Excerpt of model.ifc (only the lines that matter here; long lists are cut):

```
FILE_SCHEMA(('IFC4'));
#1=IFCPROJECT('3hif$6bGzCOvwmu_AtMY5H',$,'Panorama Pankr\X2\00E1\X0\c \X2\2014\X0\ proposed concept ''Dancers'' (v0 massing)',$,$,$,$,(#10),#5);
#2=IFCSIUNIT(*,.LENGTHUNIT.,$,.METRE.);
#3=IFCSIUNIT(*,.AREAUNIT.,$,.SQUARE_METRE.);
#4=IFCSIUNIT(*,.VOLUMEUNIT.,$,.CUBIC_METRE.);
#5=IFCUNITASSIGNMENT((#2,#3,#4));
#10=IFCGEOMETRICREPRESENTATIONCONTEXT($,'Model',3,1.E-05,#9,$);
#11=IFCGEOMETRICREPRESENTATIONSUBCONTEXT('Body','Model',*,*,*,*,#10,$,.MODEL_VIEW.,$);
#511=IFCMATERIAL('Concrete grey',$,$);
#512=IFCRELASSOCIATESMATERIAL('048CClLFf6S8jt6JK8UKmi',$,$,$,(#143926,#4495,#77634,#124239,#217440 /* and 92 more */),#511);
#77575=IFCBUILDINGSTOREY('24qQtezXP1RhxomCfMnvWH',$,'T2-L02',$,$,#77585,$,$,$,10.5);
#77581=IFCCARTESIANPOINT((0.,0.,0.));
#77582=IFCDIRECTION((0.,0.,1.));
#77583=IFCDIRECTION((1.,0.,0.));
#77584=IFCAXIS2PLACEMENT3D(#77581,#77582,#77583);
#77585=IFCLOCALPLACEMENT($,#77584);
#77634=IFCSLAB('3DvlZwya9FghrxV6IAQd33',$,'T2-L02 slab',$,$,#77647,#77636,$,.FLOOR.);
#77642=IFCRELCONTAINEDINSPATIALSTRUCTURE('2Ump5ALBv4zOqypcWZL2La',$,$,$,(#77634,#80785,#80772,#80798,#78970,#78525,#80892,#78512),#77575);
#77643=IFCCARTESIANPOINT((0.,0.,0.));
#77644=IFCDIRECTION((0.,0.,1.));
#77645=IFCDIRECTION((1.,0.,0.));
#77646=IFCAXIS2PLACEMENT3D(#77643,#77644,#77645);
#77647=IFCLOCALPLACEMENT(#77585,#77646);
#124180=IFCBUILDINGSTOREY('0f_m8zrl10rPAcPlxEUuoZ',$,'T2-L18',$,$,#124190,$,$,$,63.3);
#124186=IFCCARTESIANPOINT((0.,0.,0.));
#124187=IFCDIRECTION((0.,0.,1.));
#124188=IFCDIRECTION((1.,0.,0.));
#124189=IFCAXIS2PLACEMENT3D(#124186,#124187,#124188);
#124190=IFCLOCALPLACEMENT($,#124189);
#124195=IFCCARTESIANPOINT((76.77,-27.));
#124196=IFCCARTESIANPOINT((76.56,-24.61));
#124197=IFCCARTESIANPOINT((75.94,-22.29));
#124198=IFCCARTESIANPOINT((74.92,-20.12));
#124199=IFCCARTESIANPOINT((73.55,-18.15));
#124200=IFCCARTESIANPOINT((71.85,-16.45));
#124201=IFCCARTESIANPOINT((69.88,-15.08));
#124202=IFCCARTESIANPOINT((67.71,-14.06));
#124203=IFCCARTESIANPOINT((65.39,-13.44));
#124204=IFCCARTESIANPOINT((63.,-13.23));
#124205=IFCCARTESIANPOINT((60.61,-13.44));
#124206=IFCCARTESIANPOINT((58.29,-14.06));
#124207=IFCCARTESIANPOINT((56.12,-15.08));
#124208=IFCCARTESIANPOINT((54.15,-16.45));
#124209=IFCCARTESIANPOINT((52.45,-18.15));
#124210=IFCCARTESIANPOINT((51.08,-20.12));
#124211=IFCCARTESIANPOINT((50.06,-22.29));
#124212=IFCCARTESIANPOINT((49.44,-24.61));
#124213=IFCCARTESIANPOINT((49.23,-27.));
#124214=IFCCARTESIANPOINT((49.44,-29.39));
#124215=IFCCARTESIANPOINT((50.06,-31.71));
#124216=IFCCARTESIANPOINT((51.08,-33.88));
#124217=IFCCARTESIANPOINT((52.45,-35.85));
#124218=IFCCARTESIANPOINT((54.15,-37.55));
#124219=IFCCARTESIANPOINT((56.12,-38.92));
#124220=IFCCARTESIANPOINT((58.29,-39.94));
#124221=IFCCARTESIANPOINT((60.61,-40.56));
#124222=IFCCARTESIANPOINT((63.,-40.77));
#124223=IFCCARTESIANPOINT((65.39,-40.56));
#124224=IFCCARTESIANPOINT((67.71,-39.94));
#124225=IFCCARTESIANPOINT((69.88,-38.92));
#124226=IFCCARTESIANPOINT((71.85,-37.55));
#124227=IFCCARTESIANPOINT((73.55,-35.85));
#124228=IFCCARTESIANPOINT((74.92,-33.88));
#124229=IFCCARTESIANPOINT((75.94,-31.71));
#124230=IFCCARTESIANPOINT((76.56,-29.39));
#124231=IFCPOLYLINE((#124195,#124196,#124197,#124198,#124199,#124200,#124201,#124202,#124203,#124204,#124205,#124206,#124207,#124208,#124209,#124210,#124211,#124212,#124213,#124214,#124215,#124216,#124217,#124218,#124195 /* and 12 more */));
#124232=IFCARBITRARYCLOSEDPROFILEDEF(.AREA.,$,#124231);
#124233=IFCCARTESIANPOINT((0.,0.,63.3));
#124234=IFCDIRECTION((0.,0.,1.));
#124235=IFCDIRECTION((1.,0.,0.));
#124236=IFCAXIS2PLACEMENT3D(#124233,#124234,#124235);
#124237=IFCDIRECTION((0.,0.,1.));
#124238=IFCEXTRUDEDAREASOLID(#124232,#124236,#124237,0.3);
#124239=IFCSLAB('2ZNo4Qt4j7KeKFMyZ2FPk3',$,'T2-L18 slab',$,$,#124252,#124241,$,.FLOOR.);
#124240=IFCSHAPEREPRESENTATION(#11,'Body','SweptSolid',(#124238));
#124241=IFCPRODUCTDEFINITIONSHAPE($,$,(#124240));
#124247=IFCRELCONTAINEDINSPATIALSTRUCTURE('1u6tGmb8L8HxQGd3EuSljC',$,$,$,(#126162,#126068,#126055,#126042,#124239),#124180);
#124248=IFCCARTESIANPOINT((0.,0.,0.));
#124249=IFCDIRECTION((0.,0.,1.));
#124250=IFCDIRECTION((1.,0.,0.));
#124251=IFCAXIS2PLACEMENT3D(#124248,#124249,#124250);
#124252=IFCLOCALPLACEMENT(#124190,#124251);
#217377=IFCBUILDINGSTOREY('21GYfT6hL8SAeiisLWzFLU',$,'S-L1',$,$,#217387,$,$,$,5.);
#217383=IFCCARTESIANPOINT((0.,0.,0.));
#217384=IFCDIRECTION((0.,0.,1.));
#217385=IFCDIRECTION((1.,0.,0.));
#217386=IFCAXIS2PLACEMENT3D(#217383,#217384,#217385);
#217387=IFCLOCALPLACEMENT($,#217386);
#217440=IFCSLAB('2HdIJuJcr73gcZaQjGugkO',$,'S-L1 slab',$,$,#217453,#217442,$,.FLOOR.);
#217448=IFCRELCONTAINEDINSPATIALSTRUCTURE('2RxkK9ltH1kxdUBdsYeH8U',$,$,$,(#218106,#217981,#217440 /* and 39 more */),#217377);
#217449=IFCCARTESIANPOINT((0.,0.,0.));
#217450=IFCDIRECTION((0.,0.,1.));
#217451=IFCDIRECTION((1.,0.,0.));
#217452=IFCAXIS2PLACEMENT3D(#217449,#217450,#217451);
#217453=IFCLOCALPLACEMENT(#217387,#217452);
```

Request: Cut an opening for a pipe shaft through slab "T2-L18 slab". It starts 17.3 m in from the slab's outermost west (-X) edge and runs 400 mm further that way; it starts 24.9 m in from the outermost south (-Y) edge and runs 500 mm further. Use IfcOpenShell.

```python
import numpy as np
import ifcopenshell
import ifcopenshell.api.feature
import ifcopenshell.api.geometry
import ifcopenshell.api.root
import ifcopenshell.geom
import ifcopenshell.util.placement
import ifcopenshell.util.representation
import ifcopenshell.util.shape
import ifcopenshell.util.unit

model = ifcopenshell.open("model.ifc")
unit_scale = ifcopenshell.util.unit.calculate_unit_scale(model)
settings = ifcopenshell.geom.settings()


def volume(element):
    """Net volume in cubic metres, openings subtracted."""
    shape = ifcopenshell.geom.create_shape(settings, element)
    return ifcopenshell.util.shape.get_volume(shape.geometry)


slab = model.by_guid("2ZNo4Qt4j7KeKFMyZ2FPk3")
before = volume(slab)

# Extent in the slab's own axes, in metres. The edges named are its -X and -Y sides.
slab_shape = ifcopenshell.geom.create_shape(settings, slab)
vertices = ifcopenshell.util.shape.get_vertices(slab_shape.geometry)
x_min, y_min, bottom = vertices.min(axis=0)
top = vertices[:, 2].max()

opening = ifcopenshell.api.root.create_entity(model, ifc_class="IfcOpeningElement", name="Pipe shaft opening", predefined_type="OPENING")
context = ifcopenshell.util.representation.get_context(model, "Model", "Body", "MODEL_VIEW")
width, depth = 0.4, 0.5
outline = [(0.0, 0.0), (width, 0.0), (width, depth), (0.0, depth), (0.0, 0.0)]
# Overshoot both faces by 50 mm so the cut is clean.
shape = ifcopenshell.api.geometry.add_slab_representation(
    model, context=context, depth=top - bottom + 0.1, polyline=outline
)
ifcopenshell.api.geometry.assign_representation(model, product=opening, representation=shape)

matrix = ifcopenshell.util.placement.get_local_placement(slab.ObjectPlacement)
matrix[:, 3] = matrix @ np.append(np.array([x_min + 17.3, y_min + 24.9, bottom - 0.05]) / unit_scale, 1.0)
ifcopenshell.api.geometry.edit_object_placement(model, product=opening, matrix=matrix, is_si=False)
ifcopenshell.api.feature.add_feature(model, feature=opening, element=slab)

after = volume(slab)

print(f"slab volume {before:.3f} -> {after:.3f} m3")

model.write("model_updated.ifc")
```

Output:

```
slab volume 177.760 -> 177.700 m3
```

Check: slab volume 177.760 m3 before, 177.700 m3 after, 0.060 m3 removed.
